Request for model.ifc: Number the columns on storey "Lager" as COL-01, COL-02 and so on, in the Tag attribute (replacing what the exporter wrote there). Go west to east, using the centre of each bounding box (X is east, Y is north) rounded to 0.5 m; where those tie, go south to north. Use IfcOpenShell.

First a look at what the model holds.

```python
import ifcopenshell
import ifcopenshell.util.element
import ifcopenshell.util.placement

model = ifcopenshell.open("model.ifc")
print(model.schema)
storey = next(s for s in model.by_type("IfcBuildingStorey") if s.Name == "Lager")
columns = [e for e in ifcopenshell.util.element.get_decomposition(storey) if e.is_a("IfcColumn")]
for e in sorted(columns, key=lambda e: e.id()):
    origin = ifcopenshell.util.placement.get_local_placement(e.ObjectPlacement)[:3, 3]
    print(e.id(), e.Tag, e.Name, origin.round(2) + 0.0, sep=" | ")
```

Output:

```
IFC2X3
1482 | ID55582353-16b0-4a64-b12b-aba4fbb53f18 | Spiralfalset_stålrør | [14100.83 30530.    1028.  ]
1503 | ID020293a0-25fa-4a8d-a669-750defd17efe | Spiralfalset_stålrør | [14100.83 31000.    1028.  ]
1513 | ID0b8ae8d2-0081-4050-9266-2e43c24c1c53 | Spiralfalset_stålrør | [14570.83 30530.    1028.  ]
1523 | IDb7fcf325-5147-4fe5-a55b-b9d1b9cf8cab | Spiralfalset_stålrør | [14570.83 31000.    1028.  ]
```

```python
import ifcopenshell
import ifcopenshell.geom
import ifcopenshell.util.element
import ifcopenshell.util.shape

model = ifcopenshell.open("model.ifc")
settings = ifcopenshell.geom.settings()
settings.set("use-world-coords", True)


def centre(element):
    shape = ifcopenshell.geom.create_shape(settings, element)
    return ifcopenshell.util.shape.get_bbox_centroid(shape.geometry)


storey = next(s for s in model.by_type("IfcBuildingStorey") if s.Name == "Lager")
columns = [e for e in ifcopenshell.util.element.get_decomposition(storey) if e.is_a("IfcColumn")]

# Insertion points can sit at a corner or the storey origin, so sort by the geometry (in metres).
centres = {e: centre(e) for e in columns}
columns.sort(key=lambda e: (round(centres[e][0] / 0.5), centres[e][1]))

for i, e in enumerate(columns, start=1):
    number = f"COL-{i:02d}"
    e.Tag = number
    print(e.id(), number)

model.write("model_edited.ifc")
```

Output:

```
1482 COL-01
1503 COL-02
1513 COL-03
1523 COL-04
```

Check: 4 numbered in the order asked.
